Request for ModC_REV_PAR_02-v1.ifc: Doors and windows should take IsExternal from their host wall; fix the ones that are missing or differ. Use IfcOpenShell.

First a look at what the model holds.

```python
import ifcopenshell
import ifcopenshell.util.element

model = ifcopenshell.open("ModC_REV_PAR_02-v1.ifc")
print(model.schema)
seen = {}
for e in model.by_type("IfcDoor") + model.by_type("IfcWindow"):
    if not e.FillsVoids:
        continue
    host = e.FillsVoids[0].RelatingOpeningElement.VoidsElements[0].RelatingBuildingElement
    own = ifcopenshell.util.element.get_pset(e, f"Pset_{e.is_a()[3:].removesuffix('StandardCase')}Common", "IsExternal")
    wall = ifcopenshell.util.element.get_pset(host, "Pset_WallCommon", "IsExternal")
    seen[e.is_a(), own, wall] = seen.get((e.is_a(), own, wall), 0) + 1
for (cls, own, wall), count in sorted(seen.items(), key=str):
    print(count, cls, "IsExternal:", own, "| host wall:", wall)
```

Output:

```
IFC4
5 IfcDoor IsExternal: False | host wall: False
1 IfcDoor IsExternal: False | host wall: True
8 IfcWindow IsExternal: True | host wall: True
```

```python
import ifcopenshell
import ifcopenshell.api.pset
import ifcopenshell.util.element

model = ifcopenshell.open("ModC_REV_PAR_02-v1.ifc")

count = 0
for ifc_class, pset_name in (("IfcDoor", "Pset_DoorCommon"), ("IfcWindow", "Pset_WindowCommon")):
    for e in model.by_type(ifc_class):
        if not e.FillsVoids:
            continue
        host = e.FillsVoids[0].RelatingOpeningElement.VoidsElements[0].RelatingBuildingElement
        external = ifcopenshell.util.element.get_pset(host, "Pset_WallCommon", "IsExternal")
        if external is None or ifcopenshell.util.element.get_pset(e, pset_name, "IsExternal") == external:
            continue
        pset = ifcopenshell.api.pset.add_pset(model, product=e, name=pset_name)
        ifcopenshell.api.pset.edit_pset(model, pset=pset, properties={"IsExternal": external})
        count += 1

print(count, "updated")

model.write("ModC_REV_PAR_02-v1-out.ifc")
```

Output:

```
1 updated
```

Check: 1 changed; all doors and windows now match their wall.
